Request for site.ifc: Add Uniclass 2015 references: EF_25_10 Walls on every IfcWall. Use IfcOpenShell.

First a look at what the model holds.

```python
import ifcopenshell

model = ifcopenshell.open("site.ifc")
print(model.schema)
print("classifications:", [c.Name for c in model.by_type("IfcClassification")])
for ifc_class in ("IfcDoor", "IfcRoof", "IfcStair", "IfcWall", "IfcWindow"):
    print(ifc_class, len(model.by_type(ifc_class)))
```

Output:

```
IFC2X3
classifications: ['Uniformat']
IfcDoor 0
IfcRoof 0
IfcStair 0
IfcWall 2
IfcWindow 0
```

```python
import ifcopenshell
import ifcopenshell.api.classification

model = ifcopenshell.open("site.ifc")

# IFC2X3 requires Source and Edition and has no link from the project to the system.
system = model.create_entity("IfcClassification", Source="NBS", Edition="2015", Name="Uniclass 2015")

codes = {
    "IfcWall": ("EF_25_10", "Walls"),
}
for ifc_class, (code, name) in codes.items():
    products = model.by_type(ifc_class)
    ifcopenshell.api.classification.add_reference(
        model, products=products, classification=system, identification=code, name=name
    )
    print(code, len(products))

model.write("site_edited.ifc")
```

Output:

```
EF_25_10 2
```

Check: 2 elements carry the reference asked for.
